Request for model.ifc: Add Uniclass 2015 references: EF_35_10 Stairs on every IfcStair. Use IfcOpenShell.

First a look at what the model holds.

```python
import ifcopenshell

model = ifcopenshell.open("model.ifc")
print(model.schema)
print("classifications:", [c.Name for c in model.by_type("IfcClassification")])
for ifc_class in ("IfcDoor", "IfcRoof", "IfcStair", "IfcWall", "IfcWindow"):
    print(ifc_class, len(model.by_type(ifc_class)))
```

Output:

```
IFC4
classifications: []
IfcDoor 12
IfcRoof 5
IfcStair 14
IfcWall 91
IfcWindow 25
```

```python
import ifcopenshell
import ifcopenshell.api.classification

model = ifcopenshell.open("model.ifc")

system = ifcopenshell.api.classification.add_classification(model, classification="Uniclass 2015")

codes = {
    "IfcStair": ("EF_35_10", "Stairs"),
}
for ifc_class, (code, name) in codes.items():
    products = model.by_type(ifc_class)
    ifcopenshell.api.classification.add_reference(
        model, products=products, classification=system, identification=code, name=name
    )
    print(code, len(products))

model.write("model_v2.ifc")
```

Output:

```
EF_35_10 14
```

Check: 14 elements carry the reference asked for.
